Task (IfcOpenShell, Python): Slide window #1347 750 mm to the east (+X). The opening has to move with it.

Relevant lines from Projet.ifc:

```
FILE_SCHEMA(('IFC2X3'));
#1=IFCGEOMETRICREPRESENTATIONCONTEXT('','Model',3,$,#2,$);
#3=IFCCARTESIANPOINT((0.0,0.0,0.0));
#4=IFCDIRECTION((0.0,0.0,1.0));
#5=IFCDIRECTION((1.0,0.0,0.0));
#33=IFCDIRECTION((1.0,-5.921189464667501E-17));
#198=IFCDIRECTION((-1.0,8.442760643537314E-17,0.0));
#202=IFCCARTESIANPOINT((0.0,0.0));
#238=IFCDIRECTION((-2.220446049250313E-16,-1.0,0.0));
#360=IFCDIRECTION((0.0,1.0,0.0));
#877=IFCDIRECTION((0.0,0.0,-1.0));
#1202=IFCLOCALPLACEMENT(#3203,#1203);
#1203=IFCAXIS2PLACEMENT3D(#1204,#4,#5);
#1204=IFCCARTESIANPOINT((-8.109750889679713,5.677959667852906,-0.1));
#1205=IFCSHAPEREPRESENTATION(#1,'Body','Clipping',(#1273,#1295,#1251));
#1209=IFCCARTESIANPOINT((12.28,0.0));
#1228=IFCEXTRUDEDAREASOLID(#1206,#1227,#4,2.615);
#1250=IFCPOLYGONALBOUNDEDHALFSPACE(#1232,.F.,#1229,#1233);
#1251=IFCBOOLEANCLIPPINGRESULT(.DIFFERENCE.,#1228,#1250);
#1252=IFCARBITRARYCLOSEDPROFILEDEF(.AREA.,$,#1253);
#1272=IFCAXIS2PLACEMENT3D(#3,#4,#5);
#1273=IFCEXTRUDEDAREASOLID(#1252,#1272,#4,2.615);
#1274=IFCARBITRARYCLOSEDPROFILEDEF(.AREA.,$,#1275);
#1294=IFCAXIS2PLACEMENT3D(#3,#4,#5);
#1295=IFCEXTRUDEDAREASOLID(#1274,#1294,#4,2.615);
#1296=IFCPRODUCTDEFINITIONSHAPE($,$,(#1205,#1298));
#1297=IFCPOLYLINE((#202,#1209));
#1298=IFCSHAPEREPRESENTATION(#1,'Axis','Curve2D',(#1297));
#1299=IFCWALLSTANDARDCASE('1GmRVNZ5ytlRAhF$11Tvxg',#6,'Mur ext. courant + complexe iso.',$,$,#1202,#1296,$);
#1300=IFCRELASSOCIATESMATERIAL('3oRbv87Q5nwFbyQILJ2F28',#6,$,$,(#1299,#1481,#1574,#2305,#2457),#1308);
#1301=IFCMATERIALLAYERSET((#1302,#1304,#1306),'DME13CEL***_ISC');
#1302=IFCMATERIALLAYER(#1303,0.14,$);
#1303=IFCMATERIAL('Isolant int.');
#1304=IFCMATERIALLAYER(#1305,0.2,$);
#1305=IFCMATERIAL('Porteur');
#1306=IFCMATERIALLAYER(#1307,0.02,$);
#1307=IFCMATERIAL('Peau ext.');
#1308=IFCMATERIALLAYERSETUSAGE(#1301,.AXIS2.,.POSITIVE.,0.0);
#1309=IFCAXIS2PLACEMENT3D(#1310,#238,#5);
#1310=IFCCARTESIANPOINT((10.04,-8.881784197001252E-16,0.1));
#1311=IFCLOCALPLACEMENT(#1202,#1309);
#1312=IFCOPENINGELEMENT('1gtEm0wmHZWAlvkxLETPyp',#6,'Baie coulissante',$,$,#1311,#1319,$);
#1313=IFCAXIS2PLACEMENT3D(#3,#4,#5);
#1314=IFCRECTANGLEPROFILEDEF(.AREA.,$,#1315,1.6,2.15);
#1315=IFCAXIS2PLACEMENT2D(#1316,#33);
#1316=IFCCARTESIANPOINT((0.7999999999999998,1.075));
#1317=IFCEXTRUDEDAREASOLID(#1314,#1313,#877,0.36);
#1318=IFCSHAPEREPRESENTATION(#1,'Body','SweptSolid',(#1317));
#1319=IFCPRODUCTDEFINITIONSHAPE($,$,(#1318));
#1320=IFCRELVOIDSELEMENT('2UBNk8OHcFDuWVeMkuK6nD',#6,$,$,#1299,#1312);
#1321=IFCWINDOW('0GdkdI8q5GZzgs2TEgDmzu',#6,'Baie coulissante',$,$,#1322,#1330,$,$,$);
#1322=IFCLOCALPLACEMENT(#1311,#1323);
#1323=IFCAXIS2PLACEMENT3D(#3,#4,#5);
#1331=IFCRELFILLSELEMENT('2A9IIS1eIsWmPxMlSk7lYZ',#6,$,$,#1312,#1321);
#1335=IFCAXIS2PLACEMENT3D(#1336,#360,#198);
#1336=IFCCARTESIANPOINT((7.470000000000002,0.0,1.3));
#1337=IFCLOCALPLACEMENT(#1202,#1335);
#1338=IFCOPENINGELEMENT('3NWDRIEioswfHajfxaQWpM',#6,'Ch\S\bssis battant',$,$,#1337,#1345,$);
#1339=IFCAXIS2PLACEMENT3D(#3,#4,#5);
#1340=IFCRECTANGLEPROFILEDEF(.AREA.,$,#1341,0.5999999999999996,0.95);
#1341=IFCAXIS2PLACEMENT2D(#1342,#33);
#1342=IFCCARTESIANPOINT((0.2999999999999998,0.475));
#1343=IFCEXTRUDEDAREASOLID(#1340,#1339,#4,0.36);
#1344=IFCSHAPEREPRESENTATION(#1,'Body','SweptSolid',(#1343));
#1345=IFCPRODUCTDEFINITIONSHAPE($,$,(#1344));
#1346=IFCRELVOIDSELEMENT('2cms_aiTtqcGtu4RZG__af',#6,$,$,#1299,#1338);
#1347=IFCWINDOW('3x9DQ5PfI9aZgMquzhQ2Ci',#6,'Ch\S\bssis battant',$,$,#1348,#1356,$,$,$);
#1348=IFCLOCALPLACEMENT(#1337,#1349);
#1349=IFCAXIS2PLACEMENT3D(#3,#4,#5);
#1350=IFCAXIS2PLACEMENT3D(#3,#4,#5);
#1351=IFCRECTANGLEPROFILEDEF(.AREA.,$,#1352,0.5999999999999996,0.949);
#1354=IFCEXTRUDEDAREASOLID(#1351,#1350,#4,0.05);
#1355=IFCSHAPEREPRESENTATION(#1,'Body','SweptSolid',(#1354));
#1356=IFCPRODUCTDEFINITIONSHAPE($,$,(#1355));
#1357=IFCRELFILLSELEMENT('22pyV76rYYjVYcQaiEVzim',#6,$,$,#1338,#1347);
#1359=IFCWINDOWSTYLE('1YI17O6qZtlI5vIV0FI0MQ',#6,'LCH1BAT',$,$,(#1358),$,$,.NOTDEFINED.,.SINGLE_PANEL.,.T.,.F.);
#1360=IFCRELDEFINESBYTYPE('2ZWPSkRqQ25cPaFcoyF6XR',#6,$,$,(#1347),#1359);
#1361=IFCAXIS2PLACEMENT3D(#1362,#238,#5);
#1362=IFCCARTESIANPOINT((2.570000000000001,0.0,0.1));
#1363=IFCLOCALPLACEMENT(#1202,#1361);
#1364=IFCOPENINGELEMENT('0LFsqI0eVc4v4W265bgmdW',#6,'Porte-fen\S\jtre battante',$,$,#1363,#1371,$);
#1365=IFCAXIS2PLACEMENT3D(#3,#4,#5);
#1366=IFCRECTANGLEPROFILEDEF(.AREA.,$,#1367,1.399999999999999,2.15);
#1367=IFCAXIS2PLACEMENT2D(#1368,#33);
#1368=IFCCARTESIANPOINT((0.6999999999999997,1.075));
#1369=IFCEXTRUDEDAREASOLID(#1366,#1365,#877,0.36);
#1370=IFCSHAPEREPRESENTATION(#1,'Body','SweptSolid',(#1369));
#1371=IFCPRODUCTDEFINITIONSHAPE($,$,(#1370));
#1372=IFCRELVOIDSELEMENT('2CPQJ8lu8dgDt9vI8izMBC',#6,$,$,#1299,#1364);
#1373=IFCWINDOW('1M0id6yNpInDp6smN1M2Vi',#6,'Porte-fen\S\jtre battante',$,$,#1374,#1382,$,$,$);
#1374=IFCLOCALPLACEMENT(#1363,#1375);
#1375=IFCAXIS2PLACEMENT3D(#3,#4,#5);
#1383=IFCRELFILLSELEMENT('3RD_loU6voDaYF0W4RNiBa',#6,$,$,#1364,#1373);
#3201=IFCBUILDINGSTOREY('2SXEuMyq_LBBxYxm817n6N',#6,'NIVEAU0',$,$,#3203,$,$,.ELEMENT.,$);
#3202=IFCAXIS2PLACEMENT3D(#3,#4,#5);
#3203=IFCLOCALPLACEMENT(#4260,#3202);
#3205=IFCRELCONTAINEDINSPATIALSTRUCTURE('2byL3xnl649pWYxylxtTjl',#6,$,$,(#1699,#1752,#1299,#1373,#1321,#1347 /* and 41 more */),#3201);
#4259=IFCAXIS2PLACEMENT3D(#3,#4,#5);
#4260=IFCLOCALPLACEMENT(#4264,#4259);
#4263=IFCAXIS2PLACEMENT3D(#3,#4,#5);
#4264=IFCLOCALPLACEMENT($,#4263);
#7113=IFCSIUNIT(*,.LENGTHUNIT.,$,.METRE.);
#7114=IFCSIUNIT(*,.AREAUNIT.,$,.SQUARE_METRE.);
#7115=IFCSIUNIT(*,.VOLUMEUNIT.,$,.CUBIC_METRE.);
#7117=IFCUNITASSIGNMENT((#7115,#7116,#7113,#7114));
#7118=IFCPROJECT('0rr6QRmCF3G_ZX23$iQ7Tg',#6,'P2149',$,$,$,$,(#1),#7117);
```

```python
import ifcopenshell
import ifcopenshell.api.geometry
import ifcopenshell.util.placement

model = ifcopenshell.open("Projet.ifc")

window = model.by_guid("3x9DQ5PfI9aZgMquzhQ2Ci")
opening = window.FillsVoids[0].RelatingOpeningElement
wall = opening.VoidsElements[0].RelatingBuildingElement

wall_matrix = ifcopenshell.util.placement.get_local_placement(wall.ObjectPlacement)
shift = wall_matrix[:3, 0] * 0.75
before = ifcopenshell.util.placement.get_local_placement(window.ObjectPlacement)[:3, 3].copy()

# The window is placed relative to its opening, so it follows when the opening moves.
matrix = ifcopenshell.util.placement.get_local_placement(opening.ObjectPlacement)
matrix[:3, 3] += shift
ifcopenshell.api.geometry.edit_object_placement(
    model, product=opening, matrix=matrix, is_si=False, should_transform_children=True
)

after = ifcopenshell.util.placement.get_local_placement(window.ObjectPlacement)[:3, 3]
print("window moved by", (after - before).round(3) + 0.0)

model.write("Projet_edited.ifc")
```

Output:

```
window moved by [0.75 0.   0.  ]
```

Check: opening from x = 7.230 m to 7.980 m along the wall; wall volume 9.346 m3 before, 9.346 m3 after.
